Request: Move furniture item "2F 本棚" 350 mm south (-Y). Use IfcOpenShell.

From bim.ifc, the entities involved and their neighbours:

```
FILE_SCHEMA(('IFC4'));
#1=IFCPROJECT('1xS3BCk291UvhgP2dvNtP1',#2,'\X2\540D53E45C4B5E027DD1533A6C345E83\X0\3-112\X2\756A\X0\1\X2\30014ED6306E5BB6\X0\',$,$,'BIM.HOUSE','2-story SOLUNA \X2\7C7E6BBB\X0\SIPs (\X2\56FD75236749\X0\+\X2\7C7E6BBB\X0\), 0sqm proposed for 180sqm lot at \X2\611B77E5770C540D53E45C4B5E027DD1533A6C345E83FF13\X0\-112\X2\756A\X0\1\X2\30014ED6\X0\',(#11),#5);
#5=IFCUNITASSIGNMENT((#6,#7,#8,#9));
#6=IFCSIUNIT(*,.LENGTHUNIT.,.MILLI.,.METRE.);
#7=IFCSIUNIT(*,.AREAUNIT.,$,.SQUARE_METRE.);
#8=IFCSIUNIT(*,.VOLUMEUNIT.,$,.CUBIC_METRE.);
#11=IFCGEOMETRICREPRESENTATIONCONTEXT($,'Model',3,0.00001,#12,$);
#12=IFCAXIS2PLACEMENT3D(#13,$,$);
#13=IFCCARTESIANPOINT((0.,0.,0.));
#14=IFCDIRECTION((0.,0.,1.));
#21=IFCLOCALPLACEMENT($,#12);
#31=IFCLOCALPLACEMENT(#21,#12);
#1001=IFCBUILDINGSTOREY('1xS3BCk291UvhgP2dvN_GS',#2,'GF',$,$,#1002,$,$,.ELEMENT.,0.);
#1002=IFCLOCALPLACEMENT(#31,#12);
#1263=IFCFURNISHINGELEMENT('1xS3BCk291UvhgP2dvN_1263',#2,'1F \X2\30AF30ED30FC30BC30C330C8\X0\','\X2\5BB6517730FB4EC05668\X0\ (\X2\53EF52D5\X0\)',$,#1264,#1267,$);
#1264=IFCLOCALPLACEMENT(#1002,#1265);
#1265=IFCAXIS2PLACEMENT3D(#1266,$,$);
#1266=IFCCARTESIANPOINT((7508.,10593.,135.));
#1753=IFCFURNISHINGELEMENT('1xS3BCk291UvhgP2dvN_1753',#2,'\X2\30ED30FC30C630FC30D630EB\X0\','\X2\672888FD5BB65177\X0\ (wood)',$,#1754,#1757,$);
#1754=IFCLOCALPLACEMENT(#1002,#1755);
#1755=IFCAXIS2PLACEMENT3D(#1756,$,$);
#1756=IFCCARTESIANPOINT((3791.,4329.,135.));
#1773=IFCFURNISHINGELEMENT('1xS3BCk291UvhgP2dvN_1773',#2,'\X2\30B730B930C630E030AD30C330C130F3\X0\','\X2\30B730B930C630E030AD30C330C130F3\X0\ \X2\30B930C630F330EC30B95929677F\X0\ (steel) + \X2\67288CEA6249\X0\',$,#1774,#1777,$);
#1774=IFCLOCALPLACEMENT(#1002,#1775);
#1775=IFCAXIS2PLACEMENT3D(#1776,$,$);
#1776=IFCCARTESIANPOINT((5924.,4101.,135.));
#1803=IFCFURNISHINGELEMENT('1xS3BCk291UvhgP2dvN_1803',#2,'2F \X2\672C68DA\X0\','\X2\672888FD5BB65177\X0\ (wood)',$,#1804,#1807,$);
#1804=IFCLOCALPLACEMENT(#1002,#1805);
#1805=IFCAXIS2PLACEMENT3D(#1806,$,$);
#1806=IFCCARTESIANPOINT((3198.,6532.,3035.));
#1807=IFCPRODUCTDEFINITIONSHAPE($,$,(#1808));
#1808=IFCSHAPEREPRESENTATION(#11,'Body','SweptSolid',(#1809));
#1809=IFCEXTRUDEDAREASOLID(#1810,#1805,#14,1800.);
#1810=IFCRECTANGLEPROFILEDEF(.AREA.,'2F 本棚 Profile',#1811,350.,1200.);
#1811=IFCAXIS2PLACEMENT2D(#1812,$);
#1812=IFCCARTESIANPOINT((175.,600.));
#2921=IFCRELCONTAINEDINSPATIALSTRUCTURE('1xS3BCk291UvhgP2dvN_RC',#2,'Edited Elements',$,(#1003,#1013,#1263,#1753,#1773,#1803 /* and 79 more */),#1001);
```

```python
import ifcopenshell
import ifcopenshell.api.geometry
import ifcopenshell.util.placement
import ifcopenshell.util.unit

model = ifcopenshell.open("bim.ifc")
unit_scale = ifcopenshell.util.unit.calculate_unit_scale(model)

item = model.by_guid("1xS3BCk291UvhgP2dvN_1803")
matrix = ifcopenshell.util.placement.get_local_placement(item.ObjectPlacement)
matrix[1, 3] -= 0.35 / unit_scale
ifcopenshell.api.geometry.edit_object_placement(model, product=item, matrix=matrix, is_si=False)

print(ifcopenshell.util.placement.get_local_placement(item.ObjectPlacement).round(3) + 0.0)

model.write("bim_rev.ifc")
```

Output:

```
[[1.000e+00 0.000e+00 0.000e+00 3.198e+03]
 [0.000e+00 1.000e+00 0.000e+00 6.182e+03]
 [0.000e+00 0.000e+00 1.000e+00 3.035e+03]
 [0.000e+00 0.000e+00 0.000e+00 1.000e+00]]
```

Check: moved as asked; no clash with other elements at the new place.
